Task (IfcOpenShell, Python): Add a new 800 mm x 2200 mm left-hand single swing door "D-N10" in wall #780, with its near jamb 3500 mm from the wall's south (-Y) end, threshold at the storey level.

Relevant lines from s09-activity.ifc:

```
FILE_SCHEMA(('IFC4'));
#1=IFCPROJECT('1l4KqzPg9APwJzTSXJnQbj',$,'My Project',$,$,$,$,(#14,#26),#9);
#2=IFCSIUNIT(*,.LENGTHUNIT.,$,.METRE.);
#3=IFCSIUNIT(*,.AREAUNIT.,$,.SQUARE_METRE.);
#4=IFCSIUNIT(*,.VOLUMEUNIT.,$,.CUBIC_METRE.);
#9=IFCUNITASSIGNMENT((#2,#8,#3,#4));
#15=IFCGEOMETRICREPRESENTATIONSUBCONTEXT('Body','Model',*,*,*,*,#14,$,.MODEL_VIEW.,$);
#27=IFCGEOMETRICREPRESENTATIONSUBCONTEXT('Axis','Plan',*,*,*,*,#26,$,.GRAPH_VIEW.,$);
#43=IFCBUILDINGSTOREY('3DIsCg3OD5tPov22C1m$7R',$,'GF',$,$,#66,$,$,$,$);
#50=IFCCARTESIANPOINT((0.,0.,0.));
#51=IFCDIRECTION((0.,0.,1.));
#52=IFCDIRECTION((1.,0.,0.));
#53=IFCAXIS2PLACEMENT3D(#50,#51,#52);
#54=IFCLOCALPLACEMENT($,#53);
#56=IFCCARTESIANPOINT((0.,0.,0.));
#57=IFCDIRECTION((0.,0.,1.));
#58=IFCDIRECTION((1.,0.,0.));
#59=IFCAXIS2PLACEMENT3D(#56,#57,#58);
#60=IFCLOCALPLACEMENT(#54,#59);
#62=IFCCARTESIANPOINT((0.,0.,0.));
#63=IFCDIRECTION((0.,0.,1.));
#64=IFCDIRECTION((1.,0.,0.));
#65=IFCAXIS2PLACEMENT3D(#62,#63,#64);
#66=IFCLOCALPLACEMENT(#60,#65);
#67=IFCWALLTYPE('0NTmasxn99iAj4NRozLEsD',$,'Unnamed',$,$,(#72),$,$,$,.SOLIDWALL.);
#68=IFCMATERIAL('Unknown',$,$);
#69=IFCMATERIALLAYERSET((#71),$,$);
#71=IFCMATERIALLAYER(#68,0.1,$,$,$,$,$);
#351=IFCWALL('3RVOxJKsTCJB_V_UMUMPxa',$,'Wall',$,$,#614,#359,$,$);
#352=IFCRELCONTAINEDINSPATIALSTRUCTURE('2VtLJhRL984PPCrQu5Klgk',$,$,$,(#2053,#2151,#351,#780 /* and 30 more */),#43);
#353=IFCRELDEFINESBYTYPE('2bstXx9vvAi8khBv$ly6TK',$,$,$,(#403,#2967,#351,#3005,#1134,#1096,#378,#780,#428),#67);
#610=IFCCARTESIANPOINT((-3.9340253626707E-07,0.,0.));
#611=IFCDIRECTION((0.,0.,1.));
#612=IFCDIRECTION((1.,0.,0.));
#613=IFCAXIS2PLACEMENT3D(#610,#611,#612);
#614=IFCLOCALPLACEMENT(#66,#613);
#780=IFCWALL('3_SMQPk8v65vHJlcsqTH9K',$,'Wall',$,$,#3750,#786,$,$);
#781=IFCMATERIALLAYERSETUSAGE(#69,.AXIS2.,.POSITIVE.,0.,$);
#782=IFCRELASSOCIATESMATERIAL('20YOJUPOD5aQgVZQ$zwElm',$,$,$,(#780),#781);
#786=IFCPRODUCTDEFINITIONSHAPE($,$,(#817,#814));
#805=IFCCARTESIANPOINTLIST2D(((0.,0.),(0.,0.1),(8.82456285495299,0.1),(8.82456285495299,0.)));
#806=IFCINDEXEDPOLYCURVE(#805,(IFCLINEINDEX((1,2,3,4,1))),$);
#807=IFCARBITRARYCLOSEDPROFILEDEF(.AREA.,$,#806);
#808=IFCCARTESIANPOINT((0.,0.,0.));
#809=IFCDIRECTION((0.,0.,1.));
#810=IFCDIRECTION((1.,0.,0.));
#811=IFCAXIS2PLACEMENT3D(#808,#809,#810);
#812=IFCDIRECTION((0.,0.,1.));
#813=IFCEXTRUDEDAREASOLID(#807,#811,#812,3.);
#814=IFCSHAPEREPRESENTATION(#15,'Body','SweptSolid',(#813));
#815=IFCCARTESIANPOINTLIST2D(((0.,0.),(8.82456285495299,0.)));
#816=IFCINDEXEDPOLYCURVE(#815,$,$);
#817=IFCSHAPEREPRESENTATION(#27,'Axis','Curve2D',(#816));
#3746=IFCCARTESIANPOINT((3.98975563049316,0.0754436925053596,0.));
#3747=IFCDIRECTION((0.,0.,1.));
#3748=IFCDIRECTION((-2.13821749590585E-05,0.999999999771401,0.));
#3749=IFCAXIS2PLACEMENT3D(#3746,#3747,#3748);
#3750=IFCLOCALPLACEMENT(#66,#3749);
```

```python
import numpy as np
import ifcopenshell
import ifcopenshell.api.feature
import ifcopenshell.api.geometry
import ifcopenshell.api.root
import ifcopenshell.api.spatial
import ifcopenshell.geom
import ifcopenshell.util.element
import ifcopenshell.util.placement
import ifcopenshell.util.representation
import ifcopenshell.util.shape
import ifcopenshell.util.unit

model = ifcopenshell.open("s09-activity.ifc")
unit_scale = ifcopenshell.util.unit.calculate_unit_scale(model)
settings = ifcopenshell.geom.settings()


def volume(element):
    """Net volume in cubic metres, openings subtracted."""
    shape = ifcopenshell.geom.create_shape(settings, element)
    return ifcopenshell.util.shape.get_volume(shape.geometry)


wall = model.by_guid("3_SMQPk8v65vHJlcsqTH9K")
storey = ifcopenshell.util.element.get_container(wall, ifc_class="IfcBuildingStorey")
context = ifcopenshell.util.representation.get_context(model, "Model", "Body", "MODEL_VIEW")
before = volume(wall)

width, height, from_end, sill = 0.8, 2.2, 3.5, 0.0  # metres

# The wall runs along its own X axis, and the end named is its -X end.
wall_shape = ifcopenshell.geom.create_shape(settings, wall)
x, y, z = ifcopenshell.util.shape.get_vertices(wall_shape.geometry).T
start = x.min() + from_end
face, thickness = float(y.min()), float(y.max() - y.min())
wall_matrix = ifcopenshell.util.placement.get_local_placement(wall.ObjectPlacement)
level = ifcopenshell.util.placement.get_local_placement(storey.ObjectPlacement)[2, 3]


def in_wall(x, y):
    """Placement at x, y metres in the wall's axes, at sill height."""
    matrix = wall_matrix.copy()
    matrix[:, 3] = wall_matrix @ np.array([x / unit_scale, y / unit_scale, 0.0, 1.0])
    matrix[2, 3] = level + sill / unit_scale
    return matrix


# Opening: a box that overshoots both wall faces by 50 mm.
opening = ifcopenshell.api.root.create_entity(model, ifc_class="IfcOpeningElement", predefined_type="OPENING")
box = ifcopenshell.api.geometry.add_wall_representation(
    model, context=context, length=width, height=height, thickness=thickness + 0.1
)
ifcopenshell.api.geometry.assign_representation(model, product=opening, representation=box)
ifcopenshell.api.geometry.edit_object_placement(model, product=opening, matrix=in_wall(start, face - 0.05), is_si=False)
ifcopenshell.api.feature.add_feature(model, feature=opening, element=wall)

door = ifcopenshell.api.root.create_entity(model, ifc_class="IfcDoor", name="D-N10", predefined_type="DOOR")
door.OverallWidth, door.OverallHeight = width / unit_scale, height / unit_scale
door.OperationType = "SINGLE_SWING_LEFT"
body = ifcopenshell.api.geometry.add_door_representation(
    model,
    context=context,
    overall_width=door.OverallWidth,
    overall_height=door.OverallHeight,
    operation_type="SINGLE_SWING_LEFT",
    lining_properties={"LiningDepth": thickness / unit_scale, "ThresholdDepth": thickness / unit_scale},
)
ifcopenshell.api.geometry.assign_representation(model, product=door, representation=body)
ifcopenshell.api.spatial.assign_container(model, products=[door], relating_structure=storey)
ifcopenshell.api.feature.add_filling(model, opening=opening, element=door)

# The lining spans the wall, so the door starts at the wall face.
ifcopenshell.api.geometry.edit_object_placement(model, product=door, matrix=in_wall(start, face), is_si=False)

after = volume(wall)

print(f"wall volume {before:.3f} -> {after:.3f} m3")

model.write("s09-activity_rev.ifc")
```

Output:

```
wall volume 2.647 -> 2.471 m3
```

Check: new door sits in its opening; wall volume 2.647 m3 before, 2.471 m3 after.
